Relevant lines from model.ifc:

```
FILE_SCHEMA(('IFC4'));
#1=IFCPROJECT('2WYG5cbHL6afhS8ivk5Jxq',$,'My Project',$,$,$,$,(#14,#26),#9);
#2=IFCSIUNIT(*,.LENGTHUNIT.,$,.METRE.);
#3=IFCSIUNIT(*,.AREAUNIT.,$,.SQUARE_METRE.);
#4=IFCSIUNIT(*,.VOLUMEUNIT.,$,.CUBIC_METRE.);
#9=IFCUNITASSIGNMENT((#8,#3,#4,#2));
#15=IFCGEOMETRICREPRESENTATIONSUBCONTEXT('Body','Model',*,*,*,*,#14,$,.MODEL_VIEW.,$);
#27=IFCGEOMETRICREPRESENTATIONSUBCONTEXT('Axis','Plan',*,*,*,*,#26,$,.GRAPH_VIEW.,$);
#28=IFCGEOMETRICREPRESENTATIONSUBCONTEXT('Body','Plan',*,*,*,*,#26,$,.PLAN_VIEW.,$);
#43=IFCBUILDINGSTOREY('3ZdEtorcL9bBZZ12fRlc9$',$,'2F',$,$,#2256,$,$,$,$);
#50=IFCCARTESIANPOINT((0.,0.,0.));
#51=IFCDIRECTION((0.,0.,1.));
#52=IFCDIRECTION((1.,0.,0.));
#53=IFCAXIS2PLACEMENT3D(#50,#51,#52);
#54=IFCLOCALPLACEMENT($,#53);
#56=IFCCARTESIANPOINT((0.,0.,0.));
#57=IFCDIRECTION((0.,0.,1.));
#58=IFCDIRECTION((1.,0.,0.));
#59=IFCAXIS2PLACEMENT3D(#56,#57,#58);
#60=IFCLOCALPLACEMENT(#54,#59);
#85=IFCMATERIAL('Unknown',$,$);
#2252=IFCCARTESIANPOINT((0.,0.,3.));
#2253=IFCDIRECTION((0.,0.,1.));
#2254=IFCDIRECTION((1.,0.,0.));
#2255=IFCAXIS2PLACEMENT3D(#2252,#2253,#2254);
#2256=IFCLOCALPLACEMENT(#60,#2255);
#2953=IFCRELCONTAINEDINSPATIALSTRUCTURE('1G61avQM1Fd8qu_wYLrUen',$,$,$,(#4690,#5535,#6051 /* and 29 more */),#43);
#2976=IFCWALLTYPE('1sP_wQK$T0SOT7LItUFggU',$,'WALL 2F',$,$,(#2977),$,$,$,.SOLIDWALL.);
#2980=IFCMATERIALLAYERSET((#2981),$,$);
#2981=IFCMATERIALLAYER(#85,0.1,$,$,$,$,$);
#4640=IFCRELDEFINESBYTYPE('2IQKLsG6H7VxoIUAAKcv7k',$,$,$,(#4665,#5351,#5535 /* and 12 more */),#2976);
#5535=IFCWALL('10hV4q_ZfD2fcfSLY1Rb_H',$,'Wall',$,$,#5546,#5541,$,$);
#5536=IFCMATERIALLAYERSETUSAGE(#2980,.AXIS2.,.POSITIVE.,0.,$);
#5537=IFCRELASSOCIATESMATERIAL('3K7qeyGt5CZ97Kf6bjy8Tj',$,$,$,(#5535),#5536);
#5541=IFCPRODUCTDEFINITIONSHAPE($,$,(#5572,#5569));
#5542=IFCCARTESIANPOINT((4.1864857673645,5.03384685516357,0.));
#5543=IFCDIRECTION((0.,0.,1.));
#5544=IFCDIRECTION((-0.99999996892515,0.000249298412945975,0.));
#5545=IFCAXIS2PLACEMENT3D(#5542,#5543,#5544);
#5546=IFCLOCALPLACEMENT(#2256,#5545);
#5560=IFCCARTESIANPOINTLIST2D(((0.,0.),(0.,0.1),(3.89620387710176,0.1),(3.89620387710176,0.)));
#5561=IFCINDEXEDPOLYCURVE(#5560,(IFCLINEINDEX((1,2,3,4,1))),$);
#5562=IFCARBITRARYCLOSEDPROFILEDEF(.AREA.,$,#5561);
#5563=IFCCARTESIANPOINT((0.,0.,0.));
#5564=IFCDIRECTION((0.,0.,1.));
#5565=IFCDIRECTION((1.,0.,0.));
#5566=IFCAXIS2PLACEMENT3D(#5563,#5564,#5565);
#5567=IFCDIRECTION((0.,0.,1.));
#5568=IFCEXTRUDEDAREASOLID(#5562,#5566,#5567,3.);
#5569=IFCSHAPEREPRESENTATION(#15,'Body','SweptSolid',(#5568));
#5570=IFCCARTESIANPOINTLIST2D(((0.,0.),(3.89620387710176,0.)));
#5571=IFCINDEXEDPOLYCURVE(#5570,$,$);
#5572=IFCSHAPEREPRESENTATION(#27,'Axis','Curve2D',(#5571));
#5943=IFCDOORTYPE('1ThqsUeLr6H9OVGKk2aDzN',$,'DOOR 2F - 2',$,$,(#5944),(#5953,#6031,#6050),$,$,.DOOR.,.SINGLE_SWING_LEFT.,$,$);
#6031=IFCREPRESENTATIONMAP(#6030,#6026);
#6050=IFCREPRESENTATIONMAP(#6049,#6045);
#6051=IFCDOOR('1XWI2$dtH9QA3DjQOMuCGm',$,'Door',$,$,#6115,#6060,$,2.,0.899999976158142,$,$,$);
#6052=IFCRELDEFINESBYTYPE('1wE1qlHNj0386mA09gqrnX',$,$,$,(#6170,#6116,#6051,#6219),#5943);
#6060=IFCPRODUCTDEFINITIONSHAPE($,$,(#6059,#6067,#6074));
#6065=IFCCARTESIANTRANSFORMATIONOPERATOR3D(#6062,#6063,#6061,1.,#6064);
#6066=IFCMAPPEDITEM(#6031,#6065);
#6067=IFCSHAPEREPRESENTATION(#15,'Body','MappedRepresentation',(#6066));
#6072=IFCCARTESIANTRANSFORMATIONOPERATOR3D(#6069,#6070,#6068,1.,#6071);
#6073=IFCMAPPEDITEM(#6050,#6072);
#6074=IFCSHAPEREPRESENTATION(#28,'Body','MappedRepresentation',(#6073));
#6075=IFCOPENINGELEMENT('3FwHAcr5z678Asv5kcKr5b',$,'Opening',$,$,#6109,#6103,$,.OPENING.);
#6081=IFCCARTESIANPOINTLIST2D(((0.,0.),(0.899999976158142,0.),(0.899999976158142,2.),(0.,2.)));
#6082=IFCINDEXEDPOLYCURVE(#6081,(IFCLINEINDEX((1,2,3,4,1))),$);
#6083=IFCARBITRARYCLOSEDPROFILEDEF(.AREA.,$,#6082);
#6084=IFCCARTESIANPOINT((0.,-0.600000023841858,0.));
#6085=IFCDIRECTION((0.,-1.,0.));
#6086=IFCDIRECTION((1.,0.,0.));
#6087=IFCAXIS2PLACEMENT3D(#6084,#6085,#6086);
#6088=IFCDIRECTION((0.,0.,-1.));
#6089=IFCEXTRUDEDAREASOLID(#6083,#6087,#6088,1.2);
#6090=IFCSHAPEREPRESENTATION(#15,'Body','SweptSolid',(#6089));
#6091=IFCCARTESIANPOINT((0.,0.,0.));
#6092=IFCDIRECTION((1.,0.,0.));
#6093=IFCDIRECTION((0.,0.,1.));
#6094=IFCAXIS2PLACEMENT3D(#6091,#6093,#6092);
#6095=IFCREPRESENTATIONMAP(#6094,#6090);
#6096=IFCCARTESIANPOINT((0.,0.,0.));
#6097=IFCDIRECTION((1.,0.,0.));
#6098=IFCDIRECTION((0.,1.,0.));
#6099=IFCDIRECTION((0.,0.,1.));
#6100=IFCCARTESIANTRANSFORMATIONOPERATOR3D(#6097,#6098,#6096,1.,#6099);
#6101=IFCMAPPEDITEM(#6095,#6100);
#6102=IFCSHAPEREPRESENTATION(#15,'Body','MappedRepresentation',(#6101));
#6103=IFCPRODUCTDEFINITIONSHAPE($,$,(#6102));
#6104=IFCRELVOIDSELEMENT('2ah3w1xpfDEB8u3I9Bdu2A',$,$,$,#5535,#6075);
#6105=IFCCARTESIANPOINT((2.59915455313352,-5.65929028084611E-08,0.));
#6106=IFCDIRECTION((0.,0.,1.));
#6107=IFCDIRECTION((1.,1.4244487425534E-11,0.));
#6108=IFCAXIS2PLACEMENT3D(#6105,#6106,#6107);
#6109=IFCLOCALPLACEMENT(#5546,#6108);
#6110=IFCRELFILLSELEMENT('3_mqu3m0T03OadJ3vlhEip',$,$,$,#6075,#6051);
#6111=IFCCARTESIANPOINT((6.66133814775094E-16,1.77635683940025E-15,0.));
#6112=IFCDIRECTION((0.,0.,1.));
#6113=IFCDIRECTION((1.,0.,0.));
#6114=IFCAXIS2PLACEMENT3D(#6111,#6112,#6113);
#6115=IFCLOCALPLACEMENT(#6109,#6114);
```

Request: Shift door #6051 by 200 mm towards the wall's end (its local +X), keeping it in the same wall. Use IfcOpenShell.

```python
import ifcopenshell
import ifcopenshell.api.geometry
import ifcopenshell.util.placement
import ifcopenshell.util.unit

model = ifcopenshell.open("model.ifc")
unit_scale = ifcopenshell.util.unit.calculate_unit_scale(model)

door = model.by_guid("1XWI2$dtH9QA3DjQOMuCGm")
opening = door.FillsVoids[0].RelatingOpeningElement
wall = opening.VoidsElements[0].RelatingBuildingElement

wall_matrix = ifcopenshell.util.placement.get_local_placement(wall.ObjectPlacement)
shift = wall_matrix[:3, 0] * 0.2 / unit_scale
before = ifcopenshell.util.placement.get_local_placement(door.ObjectPlacement)[:3, 3].copy()

# The door is placed relative to its opening, so it follows when the opening moves.
matrix = ifcopenshell.util.placement.get_local_placement(opening.ObjectPlacement)
matrix[:3, 3] += shift
ifcopenshell.api.geometry.edit_object_placement(
    model, product=opening, matrix=matrix, is_si=False, should_transform_children=True
)

after = ifcopenshell.util.placement.get_local_placement(door.ObjectPlacement)[:3, 3]
print("door moved by", (after - before).round(3) + 0.0)

model.write("model-out.ifc")
```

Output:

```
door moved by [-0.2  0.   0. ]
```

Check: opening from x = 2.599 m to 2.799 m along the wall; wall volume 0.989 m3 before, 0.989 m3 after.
